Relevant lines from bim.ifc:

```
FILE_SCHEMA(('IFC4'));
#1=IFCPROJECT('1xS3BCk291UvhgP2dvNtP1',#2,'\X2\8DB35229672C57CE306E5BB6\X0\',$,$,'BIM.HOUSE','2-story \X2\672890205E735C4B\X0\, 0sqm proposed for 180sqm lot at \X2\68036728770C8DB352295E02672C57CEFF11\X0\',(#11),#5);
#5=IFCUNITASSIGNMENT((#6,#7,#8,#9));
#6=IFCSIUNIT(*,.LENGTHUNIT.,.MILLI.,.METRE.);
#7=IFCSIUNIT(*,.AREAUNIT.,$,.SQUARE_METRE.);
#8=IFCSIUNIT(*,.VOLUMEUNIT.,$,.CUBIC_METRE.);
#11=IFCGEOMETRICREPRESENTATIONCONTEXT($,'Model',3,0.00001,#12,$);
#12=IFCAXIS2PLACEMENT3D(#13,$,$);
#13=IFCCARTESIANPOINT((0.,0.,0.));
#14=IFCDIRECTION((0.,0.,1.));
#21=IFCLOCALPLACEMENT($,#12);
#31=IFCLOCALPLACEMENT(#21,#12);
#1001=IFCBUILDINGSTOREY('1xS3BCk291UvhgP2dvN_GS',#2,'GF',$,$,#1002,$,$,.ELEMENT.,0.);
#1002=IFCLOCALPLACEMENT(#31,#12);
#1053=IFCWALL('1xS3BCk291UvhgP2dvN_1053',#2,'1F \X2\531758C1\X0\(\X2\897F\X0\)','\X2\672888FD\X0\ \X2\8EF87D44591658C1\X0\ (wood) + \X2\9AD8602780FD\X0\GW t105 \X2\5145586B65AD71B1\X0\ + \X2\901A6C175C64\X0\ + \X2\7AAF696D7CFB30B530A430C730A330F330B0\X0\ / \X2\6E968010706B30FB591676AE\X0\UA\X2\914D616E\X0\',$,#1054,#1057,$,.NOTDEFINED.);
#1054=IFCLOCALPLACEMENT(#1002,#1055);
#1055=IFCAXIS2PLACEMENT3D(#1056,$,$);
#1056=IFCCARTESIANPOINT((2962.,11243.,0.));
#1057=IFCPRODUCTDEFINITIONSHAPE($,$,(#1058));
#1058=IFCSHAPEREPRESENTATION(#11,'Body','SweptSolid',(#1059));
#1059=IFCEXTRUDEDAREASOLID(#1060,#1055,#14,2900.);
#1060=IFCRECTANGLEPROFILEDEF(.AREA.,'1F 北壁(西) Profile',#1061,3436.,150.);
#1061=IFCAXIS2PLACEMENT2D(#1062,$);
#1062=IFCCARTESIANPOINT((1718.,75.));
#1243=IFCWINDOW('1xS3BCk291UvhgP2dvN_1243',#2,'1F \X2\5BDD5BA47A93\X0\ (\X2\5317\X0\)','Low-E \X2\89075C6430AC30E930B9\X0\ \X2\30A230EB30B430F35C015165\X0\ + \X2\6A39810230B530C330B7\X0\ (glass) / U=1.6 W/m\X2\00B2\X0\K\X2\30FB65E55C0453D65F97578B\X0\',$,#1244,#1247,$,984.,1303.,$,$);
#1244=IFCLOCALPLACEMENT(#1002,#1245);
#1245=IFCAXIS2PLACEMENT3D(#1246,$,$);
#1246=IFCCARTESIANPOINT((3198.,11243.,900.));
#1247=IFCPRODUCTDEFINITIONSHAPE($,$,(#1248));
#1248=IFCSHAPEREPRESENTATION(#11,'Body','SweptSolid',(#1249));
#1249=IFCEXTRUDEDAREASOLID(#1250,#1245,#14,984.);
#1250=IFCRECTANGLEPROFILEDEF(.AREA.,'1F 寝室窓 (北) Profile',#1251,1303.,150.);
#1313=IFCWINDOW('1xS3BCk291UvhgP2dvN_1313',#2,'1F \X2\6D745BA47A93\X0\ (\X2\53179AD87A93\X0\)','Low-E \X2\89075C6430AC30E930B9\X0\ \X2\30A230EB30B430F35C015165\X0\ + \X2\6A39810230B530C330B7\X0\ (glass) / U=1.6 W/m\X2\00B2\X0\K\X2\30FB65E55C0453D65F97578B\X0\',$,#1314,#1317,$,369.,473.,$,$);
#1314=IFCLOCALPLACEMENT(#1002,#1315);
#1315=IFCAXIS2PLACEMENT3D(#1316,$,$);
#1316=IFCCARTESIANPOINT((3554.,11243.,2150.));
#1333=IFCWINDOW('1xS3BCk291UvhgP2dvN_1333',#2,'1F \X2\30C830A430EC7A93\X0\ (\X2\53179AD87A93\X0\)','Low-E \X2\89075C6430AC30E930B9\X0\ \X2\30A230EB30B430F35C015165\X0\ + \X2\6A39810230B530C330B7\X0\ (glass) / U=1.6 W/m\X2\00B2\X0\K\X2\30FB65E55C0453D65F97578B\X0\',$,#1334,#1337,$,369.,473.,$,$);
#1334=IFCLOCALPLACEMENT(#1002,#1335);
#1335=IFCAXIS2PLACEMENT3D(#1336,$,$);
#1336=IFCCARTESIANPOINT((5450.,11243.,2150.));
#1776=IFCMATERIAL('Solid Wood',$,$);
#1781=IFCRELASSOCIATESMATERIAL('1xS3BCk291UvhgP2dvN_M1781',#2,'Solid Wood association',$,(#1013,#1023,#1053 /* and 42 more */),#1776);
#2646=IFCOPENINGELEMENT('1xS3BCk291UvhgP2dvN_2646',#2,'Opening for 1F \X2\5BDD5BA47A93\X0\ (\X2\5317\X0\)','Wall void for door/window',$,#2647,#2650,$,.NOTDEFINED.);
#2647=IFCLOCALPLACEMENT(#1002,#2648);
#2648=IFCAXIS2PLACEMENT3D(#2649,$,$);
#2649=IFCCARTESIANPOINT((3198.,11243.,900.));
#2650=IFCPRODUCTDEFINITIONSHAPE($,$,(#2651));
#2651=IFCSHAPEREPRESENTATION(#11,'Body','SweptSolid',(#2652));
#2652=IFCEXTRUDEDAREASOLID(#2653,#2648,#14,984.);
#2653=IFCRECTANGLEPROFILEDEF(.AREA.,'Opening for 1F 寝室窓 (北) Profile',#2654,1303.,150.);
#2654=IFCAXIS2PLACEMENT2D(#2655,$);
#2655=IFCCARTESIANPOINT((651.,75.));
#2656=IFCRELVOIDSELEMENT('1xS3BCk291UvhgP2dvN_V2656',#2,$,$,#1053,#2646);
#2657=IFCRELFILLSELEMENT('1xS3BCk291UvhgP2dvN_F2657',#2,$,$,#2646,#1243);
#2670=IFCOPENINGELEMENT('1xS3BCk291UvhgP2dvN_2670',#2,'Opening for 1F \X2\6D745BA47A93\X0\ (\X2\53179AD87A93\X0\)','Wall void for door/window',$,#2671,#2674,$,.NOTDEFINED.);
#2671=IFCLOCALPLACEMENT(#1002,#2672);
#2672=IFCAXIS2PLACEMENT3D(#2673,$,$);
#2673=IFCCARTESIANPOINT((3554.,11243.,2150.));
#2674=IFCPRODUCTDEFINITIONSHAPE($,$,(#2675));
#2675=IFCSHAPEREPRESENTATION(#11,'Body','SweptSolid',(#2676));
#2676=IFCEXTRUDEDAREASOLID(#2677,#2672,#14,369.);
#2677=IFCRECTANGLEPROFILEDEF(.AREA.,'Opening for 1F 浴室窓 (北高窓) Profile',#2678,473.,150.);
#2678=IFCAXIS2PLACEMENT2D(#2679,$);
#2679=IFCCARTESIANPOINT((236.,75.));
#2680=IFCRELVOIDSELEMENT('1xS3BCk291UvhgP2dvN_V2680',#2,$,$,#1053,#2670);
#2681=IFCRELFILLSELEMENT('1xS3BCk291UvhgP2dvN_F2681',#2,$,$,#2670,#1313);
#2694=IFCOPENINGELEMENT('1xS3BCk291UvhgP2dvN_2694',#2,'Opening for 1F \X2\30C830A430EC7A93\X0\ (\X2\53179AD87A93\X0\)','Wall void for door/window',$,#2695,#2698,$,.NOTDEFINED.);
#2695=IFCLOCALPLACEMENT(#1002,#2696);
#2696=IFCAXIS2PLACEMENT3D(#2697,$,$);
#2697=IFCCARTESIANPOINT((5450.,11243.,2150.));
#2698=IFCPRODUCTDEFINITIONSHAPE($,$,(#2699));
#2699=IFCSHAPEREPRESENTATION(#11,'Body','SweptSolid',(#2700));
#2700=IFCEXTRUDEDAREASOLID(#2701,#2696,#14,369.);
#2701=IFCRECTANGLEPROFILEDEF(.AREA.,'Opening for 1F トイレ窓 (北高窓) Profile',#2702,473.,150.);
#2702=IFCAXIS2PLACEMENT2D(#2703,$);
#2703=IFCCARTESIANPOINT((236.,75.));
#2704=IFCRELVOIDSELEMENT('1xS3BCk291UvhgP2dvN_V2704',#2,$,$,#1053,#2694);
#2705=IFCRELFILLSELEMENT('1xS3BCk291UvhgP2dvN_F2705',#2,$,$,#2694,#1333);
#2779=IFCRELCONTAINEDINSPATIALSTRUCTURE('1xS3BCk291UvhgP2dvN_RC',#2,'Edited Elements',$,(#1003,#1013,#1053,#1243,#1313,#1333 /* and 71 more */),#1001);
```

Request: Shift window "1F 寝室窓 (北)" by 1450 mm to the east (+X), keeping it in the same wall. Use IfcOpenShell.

```python
import ifcopenshell
import ifcopenshell.api.geometry
import ifcopenshell.util.placement
import ifcopenshell.util.unit

model = ifcopenshell.open("bim.ifc")
unit_scale = ifcopenshell.util.unit.calculate_unit_scale(model)

window = model.by_id(1243)
opening = window.FillsVoids[0].RelatingOpeningElement
wall = opening.VoidsElements[0].RelatingBuildingElement

wall_matrix = ifcopenshell.util.placement.get_local_placement(wall.ObjectPlacement)
shift = wall_matrix[:3, 0] * 1.45 / unit_scale
before = ifcopenshell.util.placement.get_local_placement(window.ObjectPlacement)[:3, 3].copy()

# The window is not placed relative to its opening, so move both.
for product in (opening, window):
    matrix = ifcopenshell.util.placement.get_local_placement(product.ObjectPlacement)
    matrix[:3, 3] += shift
    ifcopenshell.api.geometry.edit_object_placement(model, product=product, matrix=matrix, is_si=False)

after = ifcopenshell.util.placement.get_local_placement(window.ObjectPlacement)[:3, 3]
print("window moved by", (after - before).round(3) + 0.0)

model.write("bim_updated.ifc")
```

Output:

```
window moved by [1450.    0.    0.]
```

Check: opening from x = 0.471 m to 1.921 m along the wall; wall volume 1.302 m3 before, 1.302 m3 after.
